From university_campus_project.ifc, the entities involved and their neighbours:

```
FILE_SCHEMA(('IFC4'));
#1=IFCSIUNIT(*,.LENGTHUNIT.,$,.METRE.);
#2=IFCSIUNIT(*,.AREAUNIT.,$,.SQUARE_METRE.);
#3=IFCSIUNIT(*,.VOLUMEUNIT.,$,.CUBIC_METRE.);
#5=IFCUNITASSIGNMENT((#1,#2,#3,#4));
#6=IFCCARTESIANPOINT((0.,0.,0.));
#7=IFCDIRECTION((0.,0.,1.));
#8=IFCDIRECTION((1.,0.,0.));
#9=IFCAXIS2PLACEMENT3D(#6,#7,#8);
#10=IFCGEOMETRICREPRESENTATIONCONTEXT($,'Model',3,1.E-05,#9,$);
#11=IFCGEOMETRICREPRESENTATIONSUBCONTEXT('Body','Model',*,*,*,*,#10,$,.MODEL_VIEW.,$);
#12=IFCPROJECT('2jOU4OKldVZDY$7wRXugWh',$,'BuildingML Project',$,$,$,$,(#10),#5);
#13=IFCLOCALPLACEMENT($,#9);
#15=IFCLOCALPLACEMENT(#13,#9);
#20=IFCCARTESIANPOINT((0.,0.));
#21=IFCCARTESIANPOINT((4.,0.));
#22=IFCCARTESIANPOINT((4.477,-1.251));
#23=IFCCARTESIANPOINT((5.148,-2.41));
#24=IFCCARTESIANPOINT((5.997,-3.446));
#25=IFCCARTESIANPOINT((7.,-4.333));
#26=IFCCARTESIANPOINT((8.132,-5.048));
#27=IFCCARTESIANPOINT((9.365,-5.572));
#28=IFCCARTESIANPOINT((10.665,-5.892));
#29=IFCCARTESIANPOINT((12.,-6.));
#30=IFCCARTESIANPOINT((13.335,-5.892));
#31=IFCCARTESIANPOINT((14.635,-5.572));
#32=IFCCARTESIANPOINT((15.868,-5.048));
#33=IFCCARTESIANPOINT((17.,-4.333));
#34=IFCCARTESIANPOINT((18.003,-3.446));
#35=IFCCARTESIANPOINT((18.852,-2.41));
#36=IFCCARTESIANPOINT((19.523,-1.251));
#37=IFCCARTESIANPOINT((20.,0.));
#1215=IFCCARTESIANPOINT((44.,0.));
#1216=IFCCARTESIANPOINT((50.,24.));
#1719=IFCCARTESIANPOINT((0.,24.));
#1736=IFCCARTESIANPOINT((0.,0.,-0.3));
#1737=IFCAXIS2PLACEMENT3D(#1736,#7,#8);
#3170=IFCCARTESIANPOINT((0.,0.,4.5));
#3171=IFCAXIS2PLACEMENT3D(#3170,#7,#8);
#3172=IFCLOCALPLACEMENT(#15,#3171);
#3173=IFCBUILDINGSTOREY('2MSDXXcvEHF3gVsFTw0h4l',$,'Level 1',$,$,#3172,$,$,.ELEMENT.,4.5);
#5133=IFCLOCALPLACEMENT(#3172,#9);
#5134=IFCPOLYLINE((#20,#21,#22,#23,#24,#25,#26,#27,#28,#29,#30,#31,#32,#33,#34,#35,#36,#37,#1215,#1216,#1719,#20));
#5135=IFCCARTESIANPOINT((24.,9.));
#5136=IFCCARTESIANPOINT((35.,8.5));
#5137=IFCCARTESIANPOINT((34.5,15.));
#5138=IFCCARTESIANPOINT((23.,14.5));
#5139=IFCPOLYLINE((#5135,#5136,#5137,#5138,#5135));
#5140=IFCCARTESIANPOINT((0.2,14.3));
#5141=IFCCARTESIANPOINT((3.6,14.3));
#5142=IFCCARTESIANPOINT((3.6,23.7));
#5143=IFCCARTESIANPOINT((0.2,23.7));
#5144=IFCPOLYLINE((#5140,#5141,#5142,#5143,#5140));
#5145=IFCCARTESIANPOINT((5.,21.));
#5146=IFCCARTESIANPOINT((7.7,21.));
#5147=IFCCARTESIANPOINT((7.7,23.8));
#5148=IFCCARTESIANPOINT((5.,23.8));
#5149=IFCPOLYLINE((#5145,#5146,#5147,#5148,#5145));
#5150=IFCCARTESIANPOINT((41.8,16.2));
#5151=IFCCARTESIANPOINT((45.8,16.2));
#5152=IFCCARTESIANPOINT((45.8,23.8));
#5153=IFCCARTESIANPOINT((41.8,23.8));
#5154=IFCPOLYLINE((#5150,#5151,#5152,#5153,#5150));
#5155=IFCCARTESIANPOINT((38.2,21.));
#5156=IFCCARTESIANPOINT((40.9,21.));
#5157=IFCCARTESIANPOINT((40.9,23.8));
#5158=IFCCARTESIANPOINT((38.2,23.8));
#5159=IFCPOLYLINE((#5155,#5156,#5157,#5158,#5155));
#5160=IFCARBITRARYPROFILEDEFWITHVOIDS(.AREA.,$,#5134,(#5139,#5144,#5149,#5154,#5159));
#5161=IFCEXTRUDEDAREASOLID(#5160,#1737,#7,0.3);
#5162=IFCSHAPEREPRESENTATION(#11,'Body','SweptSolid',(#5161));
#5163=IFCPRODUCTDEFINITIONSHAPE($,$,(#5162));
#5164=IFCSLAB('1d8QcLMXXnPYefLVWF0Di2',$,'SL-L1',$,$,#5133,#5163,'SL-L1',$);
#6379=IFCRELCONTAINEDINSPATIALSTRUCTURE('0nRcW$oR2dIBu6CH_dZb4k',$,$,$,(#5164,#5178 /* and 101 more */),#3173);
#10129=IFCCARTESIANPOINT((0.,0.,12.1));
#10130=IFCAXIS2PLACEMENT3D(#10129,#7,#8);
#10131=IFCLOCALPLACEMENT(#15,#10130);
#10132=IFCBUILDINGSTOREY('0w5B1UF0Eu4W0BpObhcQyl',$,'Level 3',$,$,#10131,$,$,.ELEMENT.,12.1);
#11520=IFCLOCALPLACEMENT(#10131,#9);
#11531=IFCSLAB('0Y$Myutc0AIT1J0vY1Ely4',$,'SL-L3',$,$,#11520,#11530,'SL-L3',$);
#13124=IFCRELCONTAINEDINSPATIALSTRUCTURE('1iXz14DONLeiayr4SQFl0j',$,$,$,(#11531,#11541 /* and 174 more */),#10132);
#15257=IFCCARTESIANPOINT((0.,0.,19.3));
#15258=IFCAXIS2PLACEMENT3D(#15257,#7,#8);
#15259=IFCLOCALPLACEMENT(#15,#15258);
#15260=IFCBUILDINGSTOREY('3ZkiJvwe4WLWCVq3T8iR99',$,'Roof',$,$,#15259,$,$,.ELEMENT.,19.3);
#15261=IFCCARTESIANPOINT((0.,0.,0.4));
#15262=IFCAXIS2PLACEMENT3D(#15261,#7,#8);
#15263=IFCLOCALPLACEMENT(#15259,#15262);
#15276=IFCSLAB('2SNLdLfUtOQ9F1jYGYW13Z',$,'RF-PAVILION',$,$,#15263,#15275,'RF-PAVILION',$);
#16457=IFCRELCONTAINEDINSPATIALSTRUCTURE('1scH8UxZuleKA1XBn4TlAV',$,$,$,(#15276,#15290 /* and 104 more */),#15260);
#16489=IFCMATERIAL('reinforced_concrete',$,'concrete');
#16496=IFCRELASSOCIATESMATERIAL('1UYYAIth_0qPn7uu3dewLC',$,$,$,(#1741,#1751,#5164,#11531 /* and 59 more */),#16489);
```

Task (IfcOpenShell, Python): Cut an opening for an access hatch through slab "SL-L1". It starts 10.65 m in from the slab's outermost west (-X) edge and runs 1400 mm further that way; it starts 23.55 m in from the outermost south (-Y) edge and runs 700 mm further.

```python
import numpy as np
import ifcopenshell
import ifcopenshell.api.feature
import ifcopenshell.api.geometry
import ifcopenshell.api.root
import ifcopenshell.geom
import ifcopenshell.util.placement
import ifcopenshell.util.representation
import ifcopenshell.util.shape
import ifcopenshell.util.unit

model = ifcopenshell.open("university_campus_project.ifc")
unit_scale = ifcopenshell.util.unit.calculate_unit_scale(model)
settings = ifcopenshell.geom.settings()


def volume(element):
    """Net volume in cubic metres, openings subtracted."""
    shape = ifcopenshell.geom.create_shape(settings, element)
    return ifcopenshell.util.shape.get_volume(shape.geometry)


slab = model.by_guid("1d8QcLMXXnPYefLVWF0Di2")
before = volume(slab)

# Extent in the slab's own axes, in metres. The edges named are its -X and -Y sides.
slab_shape = ifcopenshell.geom.create_shape(settings, slab)
vertices = ifcopenshell.util.shape.get_vertices(slab_shape.geometry)
x_min, y_min, bottom = vertices.min(axis=0)
top = vertices[:, 2].max()

opening = ifcopenshell.api.root.create_entity(model, ifc_class="IfcOpeningElement", name="Access hatch opening", predefined_type="OPENING")
context = ifcopenshell.util.representation.get_context(model, "Model", "Body", "MODEL_VIEW")
width, depth = 1.4, 0.7
outline = [(0.0, 0.0), (width, 0.0), (width, depth), (0.0, depth), (0.0, 0.0)]
# Overshoot both faces by 50 mm so the cut is clean.
shape = ifcopenshell.api.geometry.add_slab_representation(
    model, context=context, depth=top - bottom + 0.1, polyline=outline
)
ifcopenshell.api.geometry.assign_representation(model, product=opening, representation=shape)

matrix = ifcopenshell.util.placement.get_local_placement(slab.ObjectPlacement)
matrix[:, 3] = matrix @ np.append(np.array([x_min + 10.65, y_min + 23.55, bottom - 0.05]) / unit_scale, 1.0)
ifcopenshell.api.geometry.edit_object_placement(model, product=opening, matrix=matrix, is_si=False)
ifcopenshell.api.feature.add_feature(model, feature=opening, element=slab)

after = volume(slab)

print(f"slab volume {before:.3f} -> {after:.3f} m3")

model.write("university_campus_project_v2.ifc")
```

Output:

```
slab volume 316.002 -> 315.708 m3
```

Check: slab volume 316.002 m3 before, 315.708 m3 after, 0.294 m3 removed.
